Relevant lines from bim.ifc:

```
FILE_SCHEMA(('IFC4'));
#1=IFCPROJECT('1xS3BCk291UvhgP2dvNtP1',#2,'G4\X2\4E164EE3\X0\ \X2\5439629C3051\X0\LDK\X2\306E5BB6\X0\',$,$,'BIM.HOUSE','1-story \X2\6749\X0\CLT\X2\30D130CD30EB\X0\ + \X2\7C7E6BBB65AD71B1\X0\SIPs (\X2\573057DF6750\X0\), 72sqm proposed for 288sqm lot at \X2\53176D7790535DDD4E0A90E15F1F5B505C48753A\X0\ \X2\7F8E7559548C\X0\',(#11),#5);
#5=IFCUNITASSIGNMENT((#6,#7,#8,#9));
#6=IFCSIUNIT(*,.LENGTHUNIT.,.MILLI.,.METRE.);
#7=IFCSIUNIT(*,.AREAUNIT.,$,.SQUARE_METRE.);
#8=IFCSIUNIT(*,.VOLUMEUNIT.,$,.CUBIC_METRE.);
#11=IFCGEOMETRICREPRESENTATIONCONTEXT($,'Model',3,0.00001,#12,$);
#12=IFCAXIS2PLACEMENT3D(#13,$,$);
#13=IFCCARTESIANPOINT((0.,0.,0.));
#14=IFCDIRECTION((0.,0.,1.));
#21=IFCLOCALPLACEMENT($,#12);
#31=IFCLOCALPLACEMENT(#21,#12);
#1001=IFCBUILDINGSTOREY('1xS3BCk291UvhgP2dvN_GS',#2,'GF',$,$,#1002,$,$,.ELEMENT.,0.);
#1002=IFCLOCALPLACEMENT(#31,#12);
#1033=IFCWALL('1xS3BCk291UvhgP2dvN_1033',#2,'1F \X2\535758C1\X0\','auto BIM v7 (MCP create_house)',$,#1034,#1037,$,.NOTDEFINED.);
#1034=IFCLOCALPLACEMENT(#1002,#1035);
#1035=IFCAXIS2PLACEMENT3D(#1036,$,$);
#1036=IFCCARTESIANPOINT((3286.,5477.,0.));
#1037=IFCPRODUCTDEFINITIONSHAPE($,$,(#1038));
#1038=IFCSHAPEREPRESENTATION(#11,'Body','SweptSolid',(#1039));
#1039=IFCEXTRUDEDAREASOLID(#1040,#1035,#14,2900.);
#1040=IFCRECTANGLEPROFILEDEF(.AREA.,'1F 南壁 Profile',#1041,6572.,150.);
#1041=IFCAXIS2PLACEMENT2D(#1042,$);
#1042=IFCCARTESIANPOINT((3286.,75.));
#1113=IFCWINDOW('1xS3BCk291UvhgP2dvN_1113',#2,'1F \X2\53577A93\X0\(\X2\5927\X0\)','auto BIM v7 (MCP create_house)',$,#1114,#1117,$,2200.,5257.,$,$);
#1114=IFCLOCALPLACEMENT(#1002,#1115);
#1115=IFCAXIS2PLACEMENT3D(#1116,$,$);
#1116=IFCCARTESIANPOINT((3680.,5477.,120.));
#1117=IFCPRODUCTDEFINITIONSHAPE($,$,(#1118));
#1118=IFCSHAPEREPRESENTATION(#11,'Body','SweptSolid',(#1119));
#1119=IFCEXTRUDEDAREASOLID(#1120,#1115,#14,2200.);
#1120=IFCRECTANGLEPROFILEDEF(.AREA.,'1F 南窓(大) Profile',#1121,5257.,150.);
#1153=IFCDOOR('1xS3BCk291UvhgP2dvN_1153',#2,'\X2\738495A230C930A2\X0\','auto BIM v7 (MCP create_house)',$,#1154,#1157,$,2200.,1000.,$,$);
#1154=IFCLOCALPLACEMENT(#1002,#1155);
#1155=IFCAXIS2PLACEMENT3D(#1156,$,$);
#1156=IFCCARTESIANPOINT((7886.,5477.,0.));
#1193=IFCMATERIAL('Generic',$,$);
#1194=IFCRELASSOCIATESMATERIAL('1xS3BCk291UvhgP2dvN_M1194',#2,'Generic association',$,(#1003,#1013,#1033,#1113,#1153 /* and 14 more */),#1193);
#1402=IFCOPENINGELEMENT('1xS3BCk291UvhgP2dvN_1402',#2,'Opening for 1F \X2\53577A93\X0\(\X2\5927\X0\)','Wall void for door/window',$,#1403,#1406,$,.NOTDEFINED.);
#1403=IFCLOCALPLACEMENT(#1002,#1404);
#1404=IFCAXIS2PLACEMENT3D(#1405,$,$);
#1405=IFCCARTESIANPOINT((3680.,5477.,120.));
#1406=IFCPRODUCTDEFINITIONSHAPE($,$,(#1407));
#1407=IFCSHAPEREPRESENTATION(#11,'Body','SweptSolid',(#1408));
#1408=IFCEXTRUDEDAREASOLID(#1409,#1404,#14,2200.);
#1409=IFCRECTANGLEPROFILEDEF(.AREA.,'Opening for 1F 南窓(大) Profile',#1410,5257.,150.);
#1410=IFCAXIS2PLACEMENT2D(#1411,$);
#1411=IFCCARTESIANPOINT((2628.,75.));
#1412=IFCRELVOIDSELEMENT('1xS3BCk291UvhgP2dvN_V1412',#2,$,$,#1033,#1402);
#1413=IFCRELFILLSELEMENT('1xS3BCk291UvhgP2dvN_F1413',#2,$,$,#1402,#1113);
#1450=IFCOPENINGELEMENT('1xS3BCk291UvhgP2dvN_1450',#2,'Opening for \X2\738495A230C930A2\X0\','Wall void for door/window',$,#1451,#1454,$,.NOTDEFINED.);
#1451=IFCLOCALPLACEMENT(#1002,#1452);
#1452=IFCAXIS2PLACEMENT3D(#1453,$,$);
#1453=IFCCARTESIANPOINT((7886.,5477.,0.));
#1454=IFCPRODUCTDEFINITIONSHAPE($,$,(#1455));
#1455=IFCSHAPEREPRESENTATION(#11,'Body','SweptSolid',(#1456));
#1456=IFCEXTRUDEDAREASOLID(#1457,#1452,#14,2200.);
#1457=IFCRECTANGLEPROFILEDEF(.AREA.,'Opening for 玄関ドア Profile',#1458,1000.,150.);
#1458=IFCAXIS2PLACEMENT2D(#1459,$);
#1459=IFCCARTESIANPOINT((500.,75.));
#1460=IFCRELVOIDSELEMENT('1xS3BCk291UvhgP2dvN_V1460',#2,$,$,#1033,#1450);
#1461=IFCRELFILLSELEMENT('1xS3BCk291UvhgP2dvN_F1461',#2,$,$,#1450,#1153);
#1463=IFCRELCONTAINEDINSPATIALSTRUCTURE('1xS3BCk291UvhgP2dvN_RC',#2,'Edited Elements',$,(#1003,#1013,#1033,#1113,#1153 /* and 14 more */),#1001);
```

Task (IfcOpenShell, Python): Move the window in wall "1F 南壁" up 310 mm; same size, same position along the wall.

```python
import numpy as np
import ifcopenshell
import ifcopenshell.api.geometry
import ifcopenshell.util.placement
import ifcopenshell.util.unit

model = ifcopenshell.open("bim.ifc")
unit_scale = ifcopenshell.util.unit.calculate_unit_scale(model)

window = model.by_id(1113)
opening = window.FillsVoids[0].RelatingOpeningElement
dz = 0.31 / unit_scale

shift = np.array([0.0, 0.0, dz])
# The window is not placed relative to its opening, so move both.
for product in (opening, window):
    matrix = ifcopenshell.util.placement.get_local_placement(product.ObjectPlacement)
    matrix[:3, 3] += shift
    ifcopenshell.api.geometry.edit_object_placement(model, product=product, matrix=matrix, is_si=False)

print(f"moved by {dz * unit_scale:+.3f} m")

model.write("bim-out.ifc")
```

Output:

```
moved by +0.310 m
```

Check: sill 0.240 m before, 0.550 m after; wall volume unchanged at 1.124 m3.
